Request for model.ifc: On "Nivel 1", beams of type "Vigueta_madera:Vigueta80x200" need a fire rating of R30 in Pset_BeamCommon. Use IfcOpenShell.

First a look at what the model holds.

```python
import ifcopenshell
import ifcopenshell.util.element

model = ifcopenshell.open("model.ifc")
print(model.schema)
storey = next(s for s in model.by_type("IfcBuildingStorey") if s.Name == "Nivel 1")
beams = [e for e in ifcopenshell.util.element.get_decomposition(storey) if e.is_a("IfcBeam")]
seen = {}
for e in beams:
    element_type = ifcopenshell.util.element.get_type(e)
    key = (element_type.Name if element_type != e and element_type else None, ifcopenshell.util.element.get_pset(e, "Pset_BeamCommon", "FireRating"))
    seen[key] = seen.get(key, 0) + 1
for (name, value), count in sorted(seen.items(), key=str):
    print(count, "x", name, "|", value)
```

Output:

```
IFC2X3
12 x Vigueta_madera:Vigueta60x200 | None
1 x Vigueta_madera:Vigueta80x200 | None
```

```python
import ifcopenshell
import ifcopenshell.api.pset
import ifcopenshell.util.element

model = ifcopenshell.open("model.ifc")

storey = next(s for s in model.by_type("IfcBuildingStorey") if s.Name == "Nivel 1")
beams = [e for e in ifcopenshell.util.element.get_decomposition(storey) if e.is_a("IfcBeam")]

count = 0
for e in beams:
    element_type = ifcopenshell.util.element.get_type(e)
    if element_type in (None, e) or element_type.Name != "Vigueta_madera:Vigueta80x200":
        continue
    # add_pset returns the element's existing set when there is one.
    pset = ifcopenshell.api.pset.add_pset(model, product=e, name="Pset_BeamCommon")
    ifcopenshell.api.pset.edit_pset(model, pset=pset, properties={"FireRating": "R30"})
    count += 1

print(count, "beams updated")

model.write("model_edited.ifc")
```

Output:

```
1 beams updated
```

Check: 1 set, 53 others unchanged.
